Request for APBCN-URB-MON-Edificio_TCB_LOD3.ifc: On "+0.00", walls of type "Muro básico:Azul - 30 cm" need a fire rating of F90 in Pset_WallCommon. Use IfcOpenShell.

First a look at what the model holds.

```python
import ifcopenshell
import ifcopenshell.util.element

model = ifcopenshell.open("APBCN-URB-MON-Edificio_TCB_LOD3.ifc")
print(model.schema)
storey = next(s for s in model.by_type("IfcBuildingStorey") if s.Name == "+0.00")
walls = [e for e in ifcopenshell.util.element.get_decomposition(storey) if e.is_a("IfcWall")]
seen = {}
for e in walls:
    element_type = ifcopenshell.util.element.get_type(e)
    key = (element_type.Name if element_type != e and element_type else None, ifcopenshell.util.element.get_pset(e, "Pset_WallCommon", "FireRating"))
    seen[key] = seen.get(key, 0) + 1
for (name, value), count in sorted(seen.items(), key=str):
    print(count, "x", name, "|", value)
```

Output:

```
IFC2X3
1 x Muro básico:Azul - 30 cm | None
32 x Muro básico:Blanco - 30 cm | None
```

```python
import ifcopenshell
import ifcopenshell.api.pset
import ifcopenshell.util.element

model = ifcopenshell.open("APBCN-URB-MON-Edificio_TCB_LOD3.ifc")

storey = next(s for s in model.by_type("IfcBuildingStorey") if s.Name == "+0.00")
walls = [e for e in ifcopenshell.util.element.get_decomposition(storey) if e.is_a("IfcWall")]

count = 0
for e in walls:
    element_type = ifcopenshell.util.element.get_type(e)
    if element_type in (None, e) or element_type.Name != "Muro básico:Azul - 30 cm":
        continue
    # add_pset returns the element's existing set when there is one.
    pset = ifcopenshell.api.pset.add_pset(model, product=e, name="Pset_WallCommon")
    ifcopenshell.api.pset.edit_pset(model, pset=pset, properties={"FireRating": "F90"})
    count += 1

print(count, "walls updated")

model.write("APBCN-URB-MON-Edificio_TCB_LOD3_v2.ifc")
```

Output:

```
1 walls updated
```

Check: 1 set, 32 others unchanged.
